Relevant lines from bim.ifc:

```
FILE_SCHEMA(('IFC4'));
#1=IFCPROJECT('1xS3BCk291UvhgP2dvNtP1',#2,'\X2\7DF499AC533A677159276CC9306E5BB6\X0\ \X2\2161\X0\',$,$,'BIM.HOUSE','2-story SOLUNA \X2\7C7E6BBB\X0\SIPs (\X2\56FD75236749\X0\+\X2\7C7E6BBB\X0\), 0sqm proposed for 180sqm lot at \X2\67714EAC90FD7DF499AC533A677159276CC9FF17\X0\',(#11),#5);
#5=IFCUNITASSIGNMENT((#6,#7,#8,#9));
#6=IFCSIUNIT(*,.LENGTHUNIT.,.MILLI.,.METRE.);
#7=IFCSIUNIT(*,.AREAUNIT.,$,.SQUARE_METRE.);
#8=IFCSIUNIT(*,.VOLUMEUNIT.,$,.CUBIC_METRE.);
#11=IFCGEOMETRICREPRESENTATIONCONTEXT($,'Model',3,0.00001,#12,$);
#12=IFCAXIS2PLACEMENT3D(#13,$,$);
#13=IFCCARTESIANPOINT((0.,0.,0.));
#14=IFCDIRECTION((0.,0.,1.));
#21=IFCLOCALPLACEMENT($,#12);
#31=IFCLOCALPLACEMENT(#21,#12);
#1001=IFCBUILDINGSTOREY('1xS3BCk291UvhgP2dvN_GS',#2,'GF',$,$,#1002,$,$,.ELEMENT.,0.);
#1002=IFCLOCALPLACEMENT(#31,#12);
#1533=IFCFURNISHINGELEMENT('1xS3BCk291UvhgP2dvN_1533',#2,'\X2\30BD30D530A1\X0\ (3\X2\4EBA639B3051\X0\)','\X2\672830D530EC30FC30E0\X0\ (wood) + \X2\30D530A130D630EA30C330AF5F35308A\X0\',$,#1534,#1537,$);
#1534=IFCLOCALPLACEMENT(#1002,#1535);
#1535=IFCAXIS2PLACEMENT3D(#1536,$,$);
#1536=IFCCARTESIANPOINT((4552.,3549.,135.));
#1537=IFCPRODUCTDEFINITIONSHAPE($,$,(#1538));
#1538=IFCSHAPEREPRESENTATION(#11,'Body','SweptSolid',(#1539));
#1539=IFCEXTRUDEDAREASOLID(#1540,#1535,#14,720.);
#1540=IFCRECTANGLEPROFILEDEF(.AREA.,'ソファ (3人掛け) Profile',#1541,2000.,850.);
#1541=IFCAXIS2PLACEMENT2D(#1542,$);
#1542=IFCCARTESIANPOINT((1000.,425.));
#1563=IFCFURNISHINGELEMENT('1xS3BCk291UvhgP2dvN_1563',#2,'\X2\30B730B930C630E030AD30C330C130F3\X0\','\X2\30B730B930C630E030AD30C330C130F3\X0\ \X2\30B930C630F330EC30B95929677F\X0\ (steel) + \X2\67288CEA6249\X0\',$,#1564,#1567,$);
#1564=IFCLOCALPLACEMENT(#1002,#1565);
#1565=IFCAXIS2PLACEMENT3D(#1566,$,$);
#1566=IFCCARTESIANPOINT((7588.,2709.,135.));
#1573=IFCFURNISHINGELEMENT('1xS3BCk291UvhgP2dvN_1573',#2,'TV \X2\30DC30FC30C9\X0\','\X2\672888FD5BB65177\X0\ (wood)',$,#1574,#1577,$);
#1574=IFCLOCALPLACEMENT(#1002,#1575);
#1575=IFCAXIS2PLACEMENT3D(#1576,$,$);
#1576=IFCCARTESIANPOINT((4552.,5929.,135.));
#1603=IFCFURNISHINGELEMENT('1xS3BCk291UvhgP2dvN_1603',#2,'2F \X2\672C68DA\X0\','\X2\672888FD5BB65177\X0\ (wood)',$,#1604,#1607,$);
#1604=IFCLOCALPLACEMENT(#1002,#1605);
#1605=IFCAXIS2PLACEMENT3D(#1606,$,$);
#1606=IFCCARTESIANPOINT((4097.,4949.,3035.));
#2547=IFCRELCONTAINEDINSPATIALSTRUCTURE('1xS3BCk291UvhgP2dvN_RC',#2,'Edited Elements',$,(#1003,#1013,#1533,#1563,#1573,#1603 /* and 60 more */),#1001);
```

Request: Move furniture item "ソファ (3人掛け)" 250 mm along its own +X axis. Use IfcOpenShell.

```python
import ifcopenshell
import ifcopenshell.api.geometry
import ifcopenshell.util.placement
import ifcopenshell.util.unit

model = ifcopenshell.open("bim.ifc")
unit_scale = ifcopenshell.util.unit.calculate_unit_scale(model)

item = model.by_guid("1xS3BCk291UvhgP2dvN_1533")
matrix = ifcopenshell.util.placement.get_local_placement(item.ObjectPlacement)
matrix[:3, 3] += matrix[:3, 0] * 0.25 / unit_scale
ifcopenshell.api.geometry.edit_object_placement(model, product=item, matrix=matrix, is_si=False)

print(ifcopenshell.util.placement.get_local_placement(item.ObjectPlacement).round(3) + 0.0)

model.write("bim-out.ifc")
```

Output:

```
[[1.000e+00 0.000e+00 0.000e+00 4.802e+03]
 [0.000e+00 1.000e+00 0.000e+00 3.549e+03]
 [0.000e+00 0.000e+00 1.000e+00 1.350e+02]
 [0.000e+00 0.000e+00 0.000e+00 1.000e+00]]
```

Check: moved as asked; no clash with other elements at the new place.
